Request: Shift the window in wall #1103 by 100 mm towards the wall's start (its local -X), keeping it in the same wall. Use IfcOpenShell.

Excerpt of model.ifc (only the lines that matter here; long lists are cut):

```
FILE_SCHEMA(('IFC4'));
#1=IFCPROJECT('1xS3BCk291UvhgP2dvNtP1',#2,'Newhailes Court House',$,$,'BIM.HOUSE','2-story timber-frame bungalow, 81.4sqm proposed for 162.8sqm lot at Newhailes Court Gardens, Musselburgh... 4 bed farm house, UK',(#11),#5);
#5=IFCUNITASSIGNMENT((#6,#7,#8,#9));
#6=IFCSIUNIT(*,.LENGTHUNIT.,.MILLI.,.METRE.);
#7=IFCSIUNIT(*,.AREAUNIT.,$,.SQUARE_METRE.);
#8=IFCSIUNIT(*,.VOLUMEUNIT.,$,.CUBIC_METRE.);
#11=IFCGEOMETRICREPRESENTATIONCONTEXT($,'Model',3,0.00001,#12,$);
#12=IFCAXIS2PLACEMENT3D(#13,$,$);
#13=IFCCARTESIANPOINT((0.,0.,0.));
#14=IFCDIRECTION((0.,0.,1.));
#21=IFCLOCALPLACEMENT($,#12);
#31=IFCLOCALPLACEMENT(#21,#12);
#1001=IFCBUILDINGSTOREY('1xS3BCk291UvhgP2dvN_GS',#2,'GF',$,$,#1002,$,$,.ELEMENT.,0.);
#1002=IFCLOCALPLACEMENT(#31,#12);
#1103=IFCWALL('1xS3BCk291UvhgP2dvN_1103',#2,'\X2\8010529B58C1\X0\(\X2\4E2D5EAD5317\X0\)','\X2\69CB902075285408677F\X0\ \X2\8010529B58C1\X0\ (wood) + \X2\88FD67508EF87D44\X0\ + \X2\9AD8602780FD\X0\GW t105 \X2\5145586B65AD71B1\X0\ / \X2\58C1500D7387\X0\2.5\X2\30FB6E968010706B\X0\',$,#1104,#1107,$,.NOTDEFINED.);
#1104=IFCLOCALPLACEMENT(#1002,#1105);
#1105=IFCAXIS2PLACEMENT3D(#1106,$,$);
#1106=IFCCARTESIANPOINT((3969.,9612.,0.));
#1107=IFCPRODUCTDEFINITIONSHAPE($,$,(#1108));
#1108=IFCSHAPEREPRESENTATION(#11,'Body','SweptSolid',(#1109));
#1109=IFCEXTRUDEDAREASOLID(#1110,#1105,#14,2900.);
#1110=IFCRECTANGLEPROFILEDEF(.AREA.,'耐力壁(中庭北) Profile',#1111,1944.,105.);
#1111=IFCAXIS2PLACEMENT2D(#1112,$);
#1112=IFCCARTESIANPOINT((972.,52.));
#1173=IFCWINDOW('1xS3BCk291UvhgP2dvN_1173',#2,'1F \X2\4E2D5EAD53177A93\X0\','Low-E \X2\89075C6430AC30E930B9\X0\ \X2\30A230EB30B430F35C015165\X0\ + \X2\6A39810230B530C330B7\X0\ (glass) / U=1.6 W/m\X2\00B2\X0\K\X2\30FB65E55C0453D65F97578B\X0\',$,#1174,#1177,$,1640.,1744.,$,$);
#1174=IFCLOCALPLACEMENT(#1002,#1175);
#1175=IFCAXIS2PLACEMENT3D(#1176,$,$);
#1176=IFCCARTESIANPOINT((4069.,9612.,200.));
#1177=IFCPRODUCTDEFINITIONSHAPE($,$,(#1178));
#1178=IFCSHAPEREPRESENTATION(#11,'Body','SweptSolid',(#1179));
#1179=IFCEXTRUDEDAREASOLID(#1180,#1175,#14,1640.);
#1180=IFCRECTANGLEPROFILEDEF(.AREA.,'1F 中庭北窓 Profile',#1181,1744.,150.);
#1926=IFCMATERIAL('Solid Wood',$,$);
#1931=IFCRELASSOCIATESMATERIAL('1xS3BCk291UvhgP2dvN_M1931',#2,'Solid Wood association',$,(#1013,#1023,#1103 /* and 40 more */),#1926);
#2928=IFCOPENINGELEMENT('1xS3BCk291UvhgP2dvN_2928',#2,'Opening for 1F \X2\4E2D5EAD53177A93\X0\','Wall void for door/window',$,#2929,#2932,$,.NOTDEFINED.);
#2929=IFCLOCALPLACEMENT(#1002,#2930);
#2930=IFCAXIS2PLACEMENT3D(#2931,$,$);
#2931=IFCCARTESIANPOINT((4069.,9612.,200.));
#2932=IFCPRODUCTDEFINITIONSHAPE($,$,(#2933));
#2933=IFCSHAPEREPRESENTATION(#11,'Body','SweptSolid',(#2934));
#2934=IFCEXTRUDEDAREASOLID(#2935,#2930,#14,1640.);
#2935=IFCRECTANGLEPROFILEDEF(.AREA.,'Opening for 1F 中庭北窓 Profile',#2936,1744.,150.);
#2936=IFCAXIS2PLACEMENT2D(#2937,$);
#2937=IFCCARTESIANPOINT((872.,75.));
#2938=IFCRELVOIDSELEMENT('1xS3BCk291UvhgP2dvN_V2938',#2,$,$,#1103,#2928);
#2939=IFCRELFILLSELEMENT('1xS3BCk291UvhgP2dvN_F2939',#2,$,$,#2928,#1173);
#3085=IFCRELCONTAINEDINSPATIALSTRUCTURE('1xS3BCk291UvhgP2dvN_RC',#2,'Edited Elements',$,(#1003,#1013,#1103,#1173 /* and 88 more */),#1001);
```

```python
import ifcopenshell
import ifcopenshell.api.geometry
import ifcopenshell.util.placement

model = ifcopenshell.open("model.ifc")

window = model.by_id(1173)
opening = window.FillsVoids[0].RelatingOpeningElement
wall = opening.VoidsElements[0].RelatingBuildingElement

wall_matrix = ifcopenshell.util.placement.get_local_placement(wall.ObjectPlacement)
shift = wall_matrix[:3, 0] * -100.0
before = ifcopenshell.util.placement.get_local_placement(window.ObjectPlacement)[:3, 3].copy()

# The window is not placed relative to its opening, so move both.
for product in (opening, window):
    matrix = ifcopenshell.util.placement.get_local_placement(product.ObjectPlacement)
    matrix[:3, 3] += shift
    ifcopenshell.api.geometry.edit_object_placement(model, product=product, matrix=matrix, is_si=False)

after = ifcopenshell.util.placement.get_local_placement(window.ObjectPlacement)[:3, 3]
print("window moved by", (after - before).round(3) + 0.0)

model.write("model_updated.ifc")
```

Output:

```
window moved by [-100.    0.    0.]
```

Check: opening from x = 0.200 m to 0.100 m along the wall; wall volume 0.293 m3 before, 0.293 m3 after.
